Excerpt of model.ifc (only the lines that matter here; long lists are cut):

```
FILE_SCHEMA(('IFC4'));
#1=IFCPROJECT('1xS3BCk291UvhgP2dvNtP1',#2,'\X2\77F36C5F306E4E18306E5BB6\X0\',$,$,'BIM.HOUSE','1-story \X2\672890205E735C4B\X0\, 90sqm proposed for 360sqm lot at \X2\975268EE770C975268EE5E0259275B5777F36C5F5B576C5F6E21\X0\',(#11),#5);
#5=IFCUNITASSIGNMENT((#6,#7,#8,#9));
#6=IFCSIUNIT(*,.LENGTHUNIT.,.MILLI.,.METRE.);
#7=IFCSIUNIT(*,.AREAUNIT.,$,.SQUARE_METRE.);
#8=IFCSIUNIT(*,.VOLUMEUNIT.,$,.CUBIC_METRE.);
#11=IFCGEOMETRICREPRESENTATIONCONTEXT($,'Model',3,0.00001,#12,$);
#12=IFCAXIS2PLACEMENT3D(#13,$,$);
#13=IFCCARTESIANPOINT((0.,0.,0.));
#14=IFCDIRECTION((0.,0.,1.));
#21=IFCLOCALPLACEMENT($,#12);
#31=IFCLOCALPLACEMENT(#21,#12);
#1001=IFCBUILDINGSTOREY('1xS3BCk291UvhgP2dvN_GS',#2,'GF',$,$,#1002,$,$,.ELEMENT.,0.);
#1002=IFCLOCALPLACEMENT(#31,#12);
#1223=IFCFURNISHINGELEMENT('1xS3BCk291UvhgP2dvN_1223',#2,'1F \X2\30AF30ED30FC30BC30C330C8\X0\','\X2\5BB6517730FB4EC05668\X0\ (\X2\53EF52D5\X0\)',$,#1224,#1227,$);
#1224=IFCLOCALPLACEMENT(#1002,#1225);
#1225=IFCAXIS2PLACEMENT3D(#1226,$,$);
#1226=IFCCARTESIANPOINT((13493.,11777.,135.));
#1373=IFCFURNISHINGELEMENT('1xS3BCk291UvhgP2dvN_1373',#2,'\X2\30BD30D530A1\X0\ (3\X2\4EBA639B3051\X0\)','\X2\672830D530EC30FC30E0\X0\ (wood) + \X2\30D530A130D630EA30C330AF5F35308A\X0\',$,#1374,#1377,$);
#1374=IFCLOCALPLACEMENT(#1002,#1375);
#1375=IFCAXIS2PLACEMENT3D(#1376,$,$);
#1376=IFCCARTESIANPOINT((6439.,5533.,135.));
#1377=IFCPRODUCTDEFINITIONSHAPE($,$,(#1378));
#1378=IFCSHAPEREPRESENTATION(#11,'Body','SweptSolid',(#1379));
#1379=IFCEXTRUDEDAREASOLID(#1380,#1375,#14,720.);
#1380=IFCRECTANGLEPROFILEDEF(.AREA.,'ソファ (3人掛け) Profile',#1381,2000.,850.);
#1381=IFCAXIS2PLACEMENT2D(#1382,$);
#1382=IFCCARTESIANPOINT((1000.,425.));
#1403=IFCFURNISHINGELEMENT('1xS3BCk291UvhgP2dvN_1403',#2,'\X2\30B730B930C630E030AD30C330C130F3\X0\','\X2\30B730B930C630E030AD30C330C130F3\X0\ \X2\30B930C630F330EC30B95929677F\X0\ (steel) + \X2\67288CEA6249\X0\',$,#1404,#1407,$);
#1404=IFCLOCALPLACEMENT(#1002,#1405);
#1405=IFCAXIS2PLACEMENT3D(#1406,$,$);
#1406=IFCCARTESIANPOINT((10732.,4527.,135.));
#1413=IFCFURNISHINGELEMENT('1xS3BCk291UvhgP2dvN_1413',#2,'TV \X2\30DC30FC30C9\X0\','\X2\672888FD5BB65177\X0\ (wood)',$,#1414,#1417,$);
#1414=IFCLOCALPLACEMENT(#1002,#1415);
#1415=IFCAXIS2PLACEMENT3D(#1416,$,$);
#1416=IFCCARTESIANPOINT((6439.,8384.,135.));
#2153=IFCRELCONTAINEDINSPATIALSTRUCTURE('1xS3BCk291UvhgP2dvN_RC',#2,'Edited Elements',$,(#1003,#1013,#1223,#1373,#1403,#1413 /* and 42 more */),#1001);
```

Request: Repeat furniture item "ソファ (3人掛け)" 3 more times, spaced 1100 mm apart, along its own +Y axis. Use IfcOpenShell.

```python
import ifcopenshell
import ifcopenshell.api.geometry
import ifcopenshell.api.root
import ifcopenshell.util.element
import ifcopenshell.util.placement
import ifcopenshell.util.unit

model = ifcopenshell.open("model.ifc")
unit_scale = ifcopenshell.util.unit.calculate_unit_scale(model)


def reuse_history(source, copy):
    """copy_class also copies each property set's owner history, people and application; keep the originals."""
    for rel in copy.IsDefinedBy:
        if rel.is_a("IfcRelDefinesByProperties") and (history := rel.RelatingPropertyDefinition.OwnerHistory):
            rel.RelatingPropertyDefinition.OwnerHistory = source.OwnerHistory
            ifcopenshell.util.element.remove_deep2(model, history)


source = model.by_guid("1xS3BCk291UvhgP2dvN_1373")
base = ifcopenshell.util.placement.get_local_placement(source.ObjectPlacement)
step = base[:3, 1] * 1.1 / unit_scale

for i in range(1, 4):
    copy = ifcopenshell.api.root.copy_class(model, product=source)
    copy.Representation = ifcopenshell.util.element.copy_deep(
        model, source.Representation, exclude=["IfcGeometricRepresentationContext", "IfcRepresentationMap"]
    )
    reuse_history(source, copy)
    matrix = base.copy()
    matrix[:3, 3] += i * step
    print("added at", matrix[:3, 3].round(3) + 0.0)
    ifcopenshell.api.geometry.edit_object_placement(model, product=copy, matrix=matrix, is_si=False)

model.write("model-out.ifc")
```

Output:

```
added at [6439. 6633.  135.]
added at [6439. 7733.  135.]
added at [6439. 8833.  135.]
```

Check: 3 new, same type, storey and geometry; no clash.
